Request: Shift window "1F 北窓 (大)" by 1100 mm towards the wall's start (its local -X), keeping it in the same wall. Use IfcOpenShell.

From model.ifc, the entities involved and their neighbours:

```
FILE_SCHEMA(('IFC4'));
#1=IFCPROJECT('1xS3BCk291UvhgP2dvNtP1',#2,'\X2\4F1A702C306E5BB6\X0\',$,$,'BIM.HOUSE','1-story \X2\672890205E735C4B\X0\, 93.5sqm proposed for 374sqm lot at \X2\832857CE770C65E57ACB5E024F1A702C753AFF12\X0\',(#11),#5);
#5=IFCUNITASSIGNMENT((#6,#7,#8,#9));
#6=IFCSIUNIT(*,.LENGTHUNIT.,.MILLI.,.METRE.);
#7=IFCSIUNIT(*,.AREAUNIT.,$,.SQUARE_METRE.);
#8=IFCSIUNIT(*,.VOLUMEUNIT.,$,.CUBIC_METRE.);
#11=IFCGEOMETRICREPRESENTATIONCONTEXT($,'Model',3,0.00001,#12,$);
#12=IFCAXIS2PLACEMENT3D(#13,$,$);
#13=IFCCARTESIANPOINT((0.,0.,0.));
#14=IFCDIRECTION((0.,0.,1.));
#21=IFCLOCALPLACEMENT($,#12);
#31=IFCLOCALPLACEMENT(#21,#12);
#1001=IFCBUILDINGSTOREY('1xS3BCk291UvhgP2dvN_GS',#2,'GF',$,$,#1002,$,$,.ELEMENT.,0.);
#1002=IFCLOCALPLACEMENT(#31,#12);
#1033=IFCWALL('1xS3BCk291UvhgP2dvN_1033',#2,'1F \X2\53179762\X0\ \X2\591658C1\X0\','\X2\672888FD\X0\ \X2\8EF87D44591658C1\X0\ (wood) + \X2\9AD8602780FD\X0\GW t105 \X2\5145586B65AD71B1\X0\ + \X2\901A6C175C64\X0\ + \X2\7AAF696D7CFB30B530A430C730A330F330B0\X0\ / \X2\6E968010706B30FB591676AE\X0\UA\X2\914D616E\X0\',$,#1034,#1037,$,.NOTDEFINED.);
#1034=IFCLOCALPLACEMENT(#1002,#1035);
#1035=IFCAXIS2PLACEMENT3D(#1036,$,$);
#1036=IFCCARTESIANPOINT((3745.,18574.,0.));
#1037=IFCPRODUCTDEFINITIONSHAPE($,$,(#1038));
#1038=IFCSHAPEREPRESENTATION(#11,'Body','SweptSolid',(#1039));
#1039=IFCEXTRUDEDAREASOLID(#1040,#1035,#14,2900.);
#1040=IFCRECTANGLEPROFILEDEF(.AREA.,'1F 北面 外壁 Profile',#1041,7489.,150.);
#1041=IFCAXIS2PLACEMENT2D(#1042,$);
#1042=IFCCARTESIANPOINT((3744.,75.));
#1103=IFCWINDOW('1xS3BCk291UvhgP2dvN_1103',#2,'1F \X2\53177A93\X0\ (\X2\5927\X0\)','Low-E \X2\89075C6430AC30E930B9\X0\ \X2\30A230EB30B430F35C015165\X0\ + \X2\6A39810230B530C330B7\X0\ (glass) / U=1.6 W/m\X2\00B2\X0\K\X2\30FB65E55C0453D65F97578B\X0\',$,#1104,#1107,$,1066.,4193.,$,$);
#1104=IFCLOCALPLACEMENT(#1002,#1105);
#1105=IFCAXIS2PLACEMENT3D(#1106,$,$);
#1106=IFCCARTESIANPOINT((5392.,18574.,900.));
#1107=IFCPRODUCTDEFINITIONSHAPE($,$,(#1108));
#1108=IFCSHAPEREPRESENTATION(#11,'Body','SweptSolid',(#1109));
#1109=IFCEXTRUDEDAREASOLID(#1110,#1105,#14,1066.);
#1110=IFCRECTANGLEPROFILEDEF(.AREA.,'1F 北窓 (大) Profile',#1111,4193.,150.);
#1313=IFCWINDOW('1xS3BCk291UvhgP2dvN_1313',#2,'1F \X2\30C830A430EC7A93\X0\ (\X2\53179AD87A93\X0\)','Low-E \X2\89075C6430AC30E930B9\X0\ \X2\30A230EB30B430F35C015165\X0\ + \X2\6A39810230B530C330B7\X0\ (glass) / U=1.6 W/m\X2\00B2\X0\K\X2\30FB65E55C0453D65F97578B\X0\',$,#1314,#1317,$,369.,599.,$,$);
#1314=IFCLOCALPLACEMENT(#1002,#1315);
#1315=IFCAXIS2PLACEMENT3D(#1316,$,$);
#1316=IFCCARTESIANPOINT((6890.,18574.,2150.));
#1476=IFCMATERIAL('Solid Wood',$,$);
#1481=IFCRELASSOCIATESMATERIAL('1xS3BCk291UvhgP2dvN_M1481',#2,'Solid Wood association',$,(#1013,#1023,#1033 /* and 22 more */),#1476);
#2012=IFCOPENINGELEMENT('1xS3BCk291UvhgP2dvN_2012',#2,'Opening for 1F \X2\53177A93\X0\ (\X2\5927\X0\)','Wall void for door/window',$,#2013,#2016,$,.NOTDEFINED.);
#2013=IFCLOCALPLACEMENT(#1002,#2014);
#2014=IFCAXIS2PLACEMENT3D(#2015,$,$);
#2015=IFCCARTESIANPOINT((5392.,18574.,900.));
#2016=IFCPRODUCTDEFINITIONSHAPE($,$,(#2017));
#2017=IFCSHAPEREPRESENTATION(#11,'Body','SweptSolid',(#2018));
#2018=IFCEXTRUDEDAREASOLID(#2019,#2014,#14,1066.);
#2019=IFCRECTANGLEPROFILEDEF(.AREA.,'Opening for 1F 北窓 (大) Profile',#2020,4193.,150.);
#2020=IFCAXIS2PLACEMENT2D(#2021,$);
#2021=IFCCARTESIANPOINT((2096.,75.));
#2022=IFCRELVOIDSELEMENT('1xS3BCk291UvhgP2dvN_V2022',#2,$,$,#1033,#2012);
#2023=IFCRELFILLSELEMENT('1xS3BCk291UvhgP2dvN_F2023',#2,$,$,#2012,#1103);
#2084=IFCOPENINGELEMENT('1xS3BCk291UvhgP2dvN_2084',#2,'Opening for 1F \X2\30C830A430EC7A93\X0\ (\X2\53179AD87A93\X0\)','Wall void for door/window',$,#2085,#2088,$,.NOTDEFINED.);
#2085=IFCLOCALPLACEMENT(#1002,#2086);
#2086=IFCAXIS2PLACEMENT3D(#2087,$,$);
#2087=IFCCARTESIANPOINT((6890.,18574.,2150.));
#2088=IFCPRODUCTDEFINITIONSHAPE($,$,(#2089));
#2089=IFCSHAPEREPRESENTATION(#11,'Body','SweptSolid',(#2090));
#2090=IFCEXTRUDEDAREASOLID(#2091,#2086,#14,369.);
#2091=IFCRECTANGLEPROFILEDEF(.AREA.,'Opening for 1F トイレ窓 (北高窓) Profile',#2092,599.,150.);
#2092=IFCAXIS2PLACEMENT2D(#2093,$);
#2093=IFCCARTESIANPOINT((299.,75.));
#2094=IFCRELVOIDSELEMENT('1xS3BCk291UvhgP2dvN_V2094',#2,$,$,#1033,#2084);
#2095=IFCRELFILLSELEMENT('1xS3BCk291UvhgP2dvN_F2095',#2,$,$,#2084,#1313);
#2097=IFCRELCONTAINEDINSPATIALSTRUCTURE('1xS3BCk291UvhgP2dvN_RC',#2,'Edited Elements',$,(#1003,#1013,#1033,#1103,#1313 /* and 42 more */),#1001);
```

```python
import ifcopenshell
import ifcopenshell.api.geometry
import ifcopenshell.util.placement
import ifcopenshell.util.unit

model = ifcopenshell.open("model.ifc")
unit_scale = ifcopenshell.util.unit.calculate_unit_scale(model)

window = model.by_id(1103)
opening = window.FillsVoids[0].RelatingOpeningElement
wall = opening.VoidsElements[0].RelatingBuildingElement

wall_matrix = ifcopenshell.util.placement.get_local_placement(wall.ObjectPlacement)
shift = wall_matrix[:3, 0] * -1.1 / unit_scale
before = ifcopenshell.util.placement.get_local_placement(window.ObjectPlacement)[:3, 3].copy()

# The window is not placed relative to its opening, so move both.
for product in (opening, window):
    matrix = ifcopenshell.util.placement.get_local_placement(product.ObjectPlacement)
    matrix[:3, 3] += shift
    ifcopenshell.api.geometry.edit_object_placement(model, product=product, matrix=matrix, is_si=False)

after = ifcopenshell.util.placement.get_local_placement(window.ObjectPlacement)[:3, 3]
print("window moved by", (after - before).round(3) + 0.0)

model.write("model-out.ifc")
```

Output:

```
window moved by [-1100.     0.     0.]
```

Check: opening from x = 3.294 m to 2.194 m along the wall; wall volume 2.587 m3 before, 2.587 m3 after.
